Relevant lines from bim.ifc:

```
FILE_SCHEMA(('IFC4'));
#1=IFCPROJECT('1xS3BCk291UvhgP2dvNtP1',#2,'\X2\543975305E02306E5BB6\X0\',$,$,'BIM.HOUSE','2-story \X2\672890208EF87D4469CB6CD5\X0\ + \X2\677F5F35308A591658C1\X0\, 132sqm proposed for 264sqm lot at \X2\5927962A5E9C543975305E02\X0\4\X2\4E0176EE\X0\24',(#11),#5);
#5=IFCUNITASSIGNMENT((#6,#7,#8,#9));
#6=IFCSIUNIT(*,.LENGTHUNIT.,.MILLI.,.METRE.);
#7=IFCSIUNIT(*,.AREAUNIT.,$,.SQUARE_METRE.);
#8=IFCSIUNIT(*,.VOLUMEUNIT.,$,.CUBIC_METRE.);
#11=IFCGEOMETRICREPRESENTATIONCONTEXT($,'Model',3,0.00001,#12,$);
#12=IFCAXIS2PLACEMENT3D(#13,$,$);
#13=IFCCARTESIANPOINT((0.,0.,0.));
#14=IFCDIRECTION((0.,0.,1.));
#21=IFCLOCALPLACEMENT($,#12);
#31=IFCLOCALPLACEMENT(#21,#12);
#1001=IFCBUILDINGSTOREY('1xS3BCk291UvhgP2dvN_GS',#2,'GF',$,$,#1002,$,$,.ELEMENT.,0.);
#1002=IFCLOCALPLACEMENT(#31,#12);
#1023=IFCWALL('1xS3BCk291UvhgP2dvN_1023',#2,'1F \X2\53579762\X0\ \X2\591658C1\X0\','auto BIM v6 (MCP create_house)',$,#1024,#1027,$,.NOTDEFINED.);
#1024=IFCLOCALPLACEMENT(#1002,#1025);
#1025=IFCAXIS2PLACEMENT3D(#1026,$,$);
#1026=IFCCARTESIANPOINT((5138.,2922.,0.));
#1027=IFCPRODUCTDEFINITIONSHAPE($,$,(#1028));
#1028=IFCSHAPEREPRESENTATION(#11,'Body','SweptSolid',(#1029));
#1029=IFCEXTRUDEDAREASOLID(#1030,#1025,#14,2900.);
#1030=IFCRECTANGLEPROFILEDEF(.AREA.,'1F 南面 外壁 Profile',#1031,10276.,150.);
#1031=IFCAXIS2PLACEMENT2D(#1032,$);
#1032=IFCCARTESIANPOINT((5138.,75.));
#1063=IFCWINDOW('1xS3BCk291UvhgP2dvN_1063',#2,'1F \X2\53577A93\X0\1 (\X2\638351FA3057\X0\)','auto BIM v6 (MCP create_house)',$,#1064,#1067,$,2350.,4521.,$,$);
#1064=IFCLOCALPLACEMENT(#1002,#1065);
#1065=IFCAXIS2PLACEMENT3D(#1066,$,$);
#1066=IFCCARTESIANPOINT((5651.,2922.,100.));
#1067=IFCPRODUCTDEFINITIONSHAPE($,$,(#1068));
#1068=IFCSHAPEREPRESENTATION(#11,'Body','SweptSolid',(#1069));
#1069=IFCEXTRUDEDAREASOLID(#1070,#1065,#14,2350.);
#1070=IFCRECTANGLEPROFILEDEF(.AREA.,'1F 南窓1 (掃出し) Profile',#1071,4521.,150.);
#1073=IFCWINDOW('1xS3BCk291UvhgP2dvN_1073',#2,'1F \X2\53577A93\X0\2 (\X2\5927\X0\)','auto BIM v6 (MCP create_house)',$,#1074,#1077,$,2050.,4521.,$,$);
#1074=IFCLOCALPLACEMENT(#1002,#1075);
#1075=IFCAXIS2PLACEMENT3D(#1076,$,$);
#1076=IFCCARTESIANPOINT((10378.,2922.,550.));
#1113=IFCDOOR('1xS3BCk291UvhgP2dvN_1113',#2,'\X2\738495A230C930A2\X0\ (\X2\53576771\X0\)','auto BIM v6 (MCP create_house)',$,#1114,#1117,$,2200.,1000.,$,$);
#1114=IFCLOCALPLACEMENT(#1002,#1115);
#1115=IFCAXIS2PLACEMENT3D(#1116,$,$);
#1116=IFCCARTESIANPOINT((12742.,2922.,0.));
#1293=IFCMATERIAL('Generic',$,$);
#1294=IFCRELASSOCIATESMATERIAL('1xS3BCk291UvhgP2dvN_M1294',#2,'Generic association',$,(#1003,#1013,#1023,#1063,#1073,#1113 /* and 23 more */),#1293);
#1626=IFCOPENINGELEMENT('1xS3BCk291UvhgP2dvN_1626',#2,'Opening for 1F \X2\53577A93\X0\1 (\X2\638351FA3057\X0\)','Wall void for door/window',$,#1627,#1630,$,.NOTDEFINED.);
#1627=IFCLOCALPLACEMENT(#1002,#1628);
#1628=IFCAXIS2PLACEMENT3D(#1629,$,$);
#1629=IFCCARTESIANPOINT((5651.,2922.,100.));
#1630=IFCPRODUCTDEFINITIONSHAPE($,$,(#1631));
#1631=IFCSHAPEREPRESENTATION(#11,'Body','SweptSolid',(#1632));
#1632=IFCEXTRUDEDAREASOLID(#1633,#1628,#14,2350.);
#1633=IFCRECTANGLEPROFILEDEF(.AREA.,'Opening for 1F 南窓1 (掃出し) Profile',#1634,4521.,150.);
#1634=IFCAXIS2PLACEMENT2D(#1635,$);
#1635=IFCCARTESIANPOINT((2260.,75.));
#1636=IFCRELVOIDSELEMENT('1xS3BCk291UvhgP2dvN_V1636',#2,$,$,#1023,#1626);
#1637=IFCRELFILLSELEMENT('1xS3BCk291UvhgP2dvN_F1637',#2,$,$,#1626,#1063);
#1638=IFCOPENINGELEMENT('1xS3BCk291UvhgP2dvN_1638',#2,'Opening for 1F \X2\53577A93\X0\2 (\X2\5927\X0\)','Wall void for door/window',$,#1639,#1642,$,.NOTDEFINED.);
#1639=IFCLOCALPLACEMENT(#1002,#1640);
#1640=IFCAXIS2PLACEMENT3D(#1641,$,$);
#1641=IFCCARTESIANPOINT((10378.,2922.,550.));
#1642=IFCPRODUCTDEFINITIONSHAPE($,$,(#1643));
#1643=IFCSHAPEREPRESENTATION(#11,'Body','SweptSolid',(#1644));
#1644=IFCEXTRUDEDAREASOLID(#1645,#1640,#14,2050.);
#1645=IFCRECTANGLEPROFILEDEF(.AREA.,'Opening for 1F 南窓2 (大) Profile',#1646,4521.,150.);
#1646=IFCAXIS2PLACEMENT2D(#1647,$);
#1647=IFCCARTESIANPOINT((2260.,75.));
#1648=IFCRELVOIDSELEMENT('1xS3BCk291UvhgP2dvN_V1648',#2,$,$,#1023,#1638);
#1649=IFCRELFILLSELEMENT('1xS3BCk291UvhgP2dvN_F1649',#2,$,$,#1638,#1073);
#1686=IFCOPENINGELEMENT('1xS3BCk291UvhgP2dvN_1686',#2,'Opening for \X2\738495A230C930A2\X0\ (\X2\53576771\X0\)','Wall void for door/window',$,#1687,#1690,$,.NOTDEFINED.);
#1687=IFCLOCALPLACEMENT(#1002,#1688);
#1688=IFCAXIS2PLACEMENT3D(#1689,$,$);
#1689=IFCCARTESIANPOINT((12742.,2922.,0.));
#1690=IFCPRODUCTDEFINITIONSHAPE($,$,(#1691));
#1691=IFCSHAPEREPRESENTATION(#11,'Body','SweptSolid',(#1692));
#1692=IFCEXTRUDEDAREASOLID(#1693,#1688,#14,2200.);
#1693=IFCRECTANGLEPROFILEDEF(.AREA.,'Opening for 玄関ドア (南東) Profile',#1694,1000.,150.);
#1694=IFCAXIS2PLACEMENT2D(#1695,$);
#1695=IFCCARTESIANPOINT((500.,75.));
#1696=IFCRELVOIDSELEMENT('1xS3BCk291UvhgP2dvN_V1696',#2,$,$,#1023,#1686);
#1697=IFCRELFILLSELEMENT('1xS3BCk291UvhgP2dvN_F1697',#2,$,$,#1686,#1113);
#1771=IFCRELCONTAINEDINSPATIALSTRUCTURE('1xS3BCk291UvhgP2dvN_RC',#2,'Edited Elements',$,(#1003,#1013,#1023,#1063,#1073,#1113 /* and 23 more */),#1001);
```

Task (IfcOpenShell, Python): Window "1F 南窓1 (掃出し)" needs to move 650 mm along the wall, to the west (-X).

```python
import ifcopenshell
import ifcopenshell.api.geometry
import ifcopenshell.util.placement
import ifcopenshell.util.unit

model = ifcopenshell.open("bim.ifc")
unit_scale = ifcopenshell.util.unit.calculate_unit_scale(model)

window = model.by_guid("1xS3BCk291UvhgP2dvN_1063")
opening = window.FillsVoids[0].RelatingOpeningElement
wall = opening.VoidsElements[0].RelatingBuildingElement

wall_matrix = ifcopenshell.util.placement.get_local_placement(wall.ObjectPlacement)
shift = wall_matrix[:3, 0] * -0.65 / unit_scale
before = ifcopenshell.util.placement.get_local_placement(window.ObjectPlacement)[:3, 3].copy()

# The window is not placed relative to its opening, so move both.
for product in (opening, window):
    matrix = ifcopenshell.util.placement.get_local_placement(product.ObjectPlacement)
    matrix[:3, 3] += shift
    ifcopenshell.api.geometry.edit_object_placement(model, product=product, matrix=matrix, is_si=False)

after = ifcopenshell.util.placement.get_local_placement(window.ObjectPlacement)[:3, 3]
print("window moved by", (after - before).round(3) + 0.0)

model.write("bim_rev.ifc")
```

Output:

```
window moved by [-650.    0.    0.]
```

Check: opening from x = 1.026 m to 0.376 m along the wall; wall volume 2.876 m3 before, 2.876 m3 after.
